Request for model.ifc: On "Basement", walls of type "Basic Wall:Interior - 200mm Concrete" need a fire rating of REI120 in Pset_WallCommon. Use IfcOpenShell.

First a look at what the model holds.

```python
import ifcopenshell
import ifcopenshell.util.element

model = ifcopenshell.open("model.ifc")
print(model.schema)
storey = next(s for s in model.by_type("IfcBuildingStorey") if s.Name == "Basement")
walls = [e for e in ifcopenshell.util.element.get_decomposition(storey) if e.is_a("IfcWall")]
seen = {}
for e in walls:
    element_type = ifcopenshell.util.element.get_type(e)
    key = (element_type.Name if element_type != e and element_type else None, ifcopenshell.util.element.get_pset(e, "Pset_WallCommon", "FireRating"))
    seen[key] = seen.get(key, 0) + 1
for (name, value), count in sorted(seen.items(), key=str):
    print(count, "x", name, "|", value)
```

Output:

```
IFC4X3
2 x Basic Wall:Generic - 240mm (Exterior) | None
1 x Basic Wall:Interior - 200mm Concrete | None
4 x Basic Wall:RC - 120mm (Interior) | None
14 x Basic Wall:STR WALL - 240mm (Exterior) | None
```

```python
import ifcopenshell
import ifcopenshell.api.pset
import ifcopenshell.util.element

model = ifcopenshell.open("model.ifc")

storey = next(s for s in model.by_type("IfcBuildingStorey") if s.Name == "Basement")
walls = [e for e in ifcopenshell.util.element.get_decomposition(storey) if e.is_a("IfcWall")]

count = 0
for e in walls:
    element_type = ifcopenshell.util.element.get_type(e)
    if element_type in (None, e) or element_type.Name != "Basic Wall:Interior - 200mm Concrete":
        continue
    # add_pset returns the element's existing set when there is one.
    pset = ifcopenshell.api.pset.add_pset(model, product=e, name="Pset_WallCommon")
    ifcopenshell.api.pset.edit_pset(model, pset=pset, properties={"FireRating": "REI120"})
    count += 1

print(count, "walls updated")

model.write("model_rev.ifc")
```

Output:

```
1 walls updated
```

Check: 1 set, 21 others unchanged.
